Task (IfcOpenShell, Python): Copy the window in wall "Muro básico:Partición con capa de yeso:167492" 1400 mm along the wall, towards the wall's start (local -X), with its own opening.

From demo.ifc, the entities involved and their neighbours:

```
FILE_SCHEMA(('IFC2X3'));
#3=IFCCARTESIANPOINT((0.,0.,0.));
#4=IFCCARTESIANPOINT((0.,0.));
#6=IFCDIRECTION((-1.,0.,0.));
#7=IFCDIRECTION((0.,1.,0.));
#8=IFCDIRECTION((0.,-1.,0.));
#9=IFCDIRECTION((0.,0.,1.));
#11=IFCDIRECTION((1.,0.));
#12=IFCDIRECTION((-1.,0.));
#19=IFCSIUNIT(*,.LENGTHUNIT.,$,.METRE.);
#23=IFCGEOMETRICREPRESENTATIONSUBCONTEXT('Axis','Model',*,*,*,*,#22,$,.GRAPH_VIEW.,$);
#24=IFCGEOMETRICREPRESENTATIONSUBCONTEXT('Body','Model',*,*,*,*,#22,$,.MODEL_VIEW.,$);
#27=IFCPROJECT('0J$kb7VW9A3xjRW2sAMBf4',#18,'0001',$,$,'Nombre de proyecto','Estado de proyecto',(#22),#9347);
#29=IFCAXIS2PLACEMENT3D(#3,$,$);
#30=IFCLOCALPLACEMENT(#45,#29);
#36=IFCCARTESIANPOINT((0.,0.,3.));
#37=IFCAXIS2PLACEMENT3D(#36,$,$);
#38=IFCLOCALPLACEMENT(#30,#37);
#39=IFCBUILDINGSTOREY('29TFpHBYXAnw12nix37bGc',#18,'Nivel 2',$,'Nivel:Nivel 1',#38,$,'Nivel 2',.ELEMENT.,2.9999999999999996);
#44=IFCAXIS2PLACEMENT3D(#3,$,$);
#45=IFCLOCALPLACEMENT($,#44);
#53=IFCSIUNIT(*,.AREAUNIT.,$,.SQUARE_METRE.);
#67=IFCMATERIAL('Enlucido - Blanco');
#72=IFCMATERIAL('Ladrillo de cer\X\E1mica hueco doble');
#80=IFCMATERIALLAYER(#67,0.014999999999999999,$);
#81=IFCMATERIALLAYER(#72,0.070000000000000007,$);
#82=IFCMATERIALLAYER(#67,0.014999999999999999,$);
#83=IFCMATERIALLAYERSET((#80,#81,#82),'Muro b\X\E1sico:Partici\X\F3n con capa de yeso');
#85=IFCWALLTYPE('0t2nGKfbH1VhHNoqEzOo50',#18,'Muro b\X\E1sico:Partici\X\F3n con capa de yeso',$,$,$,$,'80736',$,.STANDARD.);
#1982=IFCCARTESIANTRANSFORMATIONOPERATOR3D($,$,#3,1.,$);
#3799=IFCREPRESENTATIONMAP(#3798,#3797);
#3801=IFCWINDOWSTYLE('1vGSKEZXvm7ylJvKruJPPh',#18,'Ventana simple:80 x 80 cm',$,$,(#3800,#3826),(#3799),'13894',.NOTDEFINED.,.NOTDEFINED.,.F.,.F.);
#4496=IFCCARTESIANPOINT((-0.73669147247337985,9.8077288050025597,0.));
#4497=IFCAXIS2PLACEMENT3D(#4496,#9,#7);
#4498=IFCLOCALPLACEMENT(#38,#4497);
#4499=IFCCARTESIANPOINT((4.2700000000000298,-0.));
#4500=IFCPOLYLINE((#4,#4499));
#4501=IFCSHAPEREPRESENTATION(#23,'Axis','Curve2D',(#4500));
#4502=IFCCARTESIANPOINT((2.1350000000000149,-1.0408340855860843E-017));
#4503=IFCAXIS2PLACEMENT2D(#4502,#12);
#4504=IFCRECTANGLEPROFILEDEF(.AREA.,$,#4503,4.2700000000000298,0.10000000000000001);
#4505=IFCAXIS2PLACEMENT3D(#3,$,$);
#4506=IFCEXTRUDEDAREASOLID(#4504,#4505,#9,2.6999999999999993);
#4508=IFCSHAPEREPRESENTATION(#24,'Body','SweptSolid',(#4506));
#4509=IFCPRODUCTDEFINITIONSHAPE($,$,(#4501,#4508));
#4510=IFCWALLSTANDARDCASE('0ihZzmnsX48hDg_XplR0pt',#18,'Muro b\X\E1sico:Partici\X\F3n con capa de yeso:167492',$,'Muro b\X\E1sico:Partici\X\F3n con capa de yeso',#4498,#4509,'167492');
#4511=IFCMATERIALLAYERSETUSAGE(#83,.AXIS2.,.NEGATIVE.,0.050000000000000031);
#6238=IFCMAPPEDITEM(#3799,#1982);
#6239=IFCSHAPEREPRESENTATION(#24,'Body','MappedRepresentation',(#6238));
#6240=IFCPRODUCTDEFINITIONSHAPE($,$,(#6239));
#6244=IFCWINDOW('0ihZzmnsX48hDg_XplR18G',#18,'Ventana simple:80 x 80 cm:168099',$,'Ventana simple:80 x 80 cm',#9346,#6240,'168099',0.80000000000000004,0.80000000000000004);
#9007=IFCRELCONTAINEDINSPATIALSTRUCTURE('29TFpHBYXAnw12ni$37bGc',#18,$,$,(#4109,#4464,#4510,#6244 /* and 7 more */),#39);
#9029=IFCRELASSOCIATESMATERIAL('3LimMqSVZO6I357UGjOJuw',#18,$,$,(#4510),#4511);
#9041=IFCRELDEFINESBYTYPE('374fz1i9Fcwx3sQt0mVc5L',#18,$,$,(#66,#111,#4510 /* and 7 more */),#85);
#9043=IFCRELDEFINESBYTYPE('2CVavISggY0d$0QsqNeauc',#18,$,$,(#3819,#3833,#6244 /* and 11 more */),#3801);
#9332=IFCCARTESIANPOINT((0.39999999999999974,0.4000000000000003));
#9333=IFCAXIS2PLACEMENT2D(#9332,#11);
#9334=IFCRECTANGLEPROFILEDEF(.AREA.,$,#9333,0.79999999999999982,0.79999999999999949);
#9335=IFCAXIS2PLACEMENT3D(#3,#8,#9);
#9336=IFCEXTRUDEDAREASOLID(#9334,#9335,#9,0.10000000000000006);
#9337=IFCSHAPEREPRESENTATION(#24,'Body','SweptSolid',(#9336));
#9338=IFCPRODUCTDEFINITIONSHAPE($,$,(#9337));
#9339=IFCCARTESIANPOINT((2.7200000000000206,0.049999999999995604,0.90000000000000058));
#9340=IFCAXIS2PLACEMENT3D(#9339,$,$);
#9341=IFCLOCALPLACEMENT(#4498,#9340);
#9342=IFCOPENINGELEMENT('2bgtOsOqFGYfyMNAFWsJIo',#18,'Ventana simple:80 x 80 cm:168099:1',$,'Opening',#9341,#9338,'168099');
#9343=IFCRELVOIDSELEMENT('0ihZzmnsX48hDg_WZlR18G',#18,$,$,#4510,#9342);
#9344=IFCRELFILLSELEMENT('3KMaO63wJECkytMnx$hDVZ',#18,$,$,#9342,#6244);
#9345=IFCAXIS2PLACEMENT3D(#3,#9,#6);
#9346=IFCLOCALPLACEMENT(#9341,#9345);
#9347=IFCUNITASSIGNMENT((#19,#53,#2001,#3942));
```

```python
import ifcopenshell
import ifcopenshell.api.feature
import ifcopenshell.api.geometry
import ifcopenshell.api.root
import ifcopenshell.geom
import ifcopenshell.util.element
import ifcopenshell.util.placement
import ifcopenshell.util.shape
import ifcopenshell.util.unit

model = ifcopenshell.open("demo.ifc")
unit_scale = ifcopenshell.util.unit.calculate_unit_scale(model)
settings = ifcopenshell.geom.settings()


def volume(element):
    """Net volume in cubic metres, openings subtracted."""
    shape = ifcopenshell.geom.create_shape(settings, element)
    return ifcopenshell.util.shape.get_volume(shape.geometry)


def reuse_history(source, copy):
    """copy_class also copies each property set's owner history, people and application; keep the originals."""
    for rel in copy.IsDefinedBy:
        if rel.is_a("IfcRelDefinesByProperties") and (history := rel.RelatingPropertyDefinition.OwnerHistory):
            rel.RelatingPropertyDefinition.OwnerHistory = source.OwnerHistory
            ifcopenshell.util.element.remove_deep2(model, history)


window = model.by_guid("0ihZzmnsX48hDg_XplR18G")
opening = window.FillsVoids[0].RelatingOpeningElement
wall = opening.VoidsElements[0].RelatingBuildingElement
before = volume(wall)
shift = ifcopenshell.util.placement.get_local_placement(wall.ObjectPlacement)[:3, 0] * -1.4 / unit_scale

# copy_class copies the void relationship, type, container and properties, but no geometry.
new_opening = ifcopenshell.api.root.copy_class(model, product=opening)
new_opening.Representation = ifcopenshell.util.element.copy_deep(
    model, opening.Representation, exclude=["IfcGeometricRepresentationContext", "IfcRepresentationMap"]
)
new_opening.Name = "Ventana simple:80 x 80 cm"
new_opening.Tag = None
new_window = ifcopenshell.api.root.copy_class(model, product=window)
new_window.Representation = ifcopenshell.util.element.copy_deep(
    model, window.Representation, exclude=["IfcGeometricRepresentationContext", "IfcRepresentationMap"]
)
new_window.Name = "Ventana simple:80 x 80 cm"
new_window.Tag = None
reuse_history(window, new_window)
fills = ifcopenshell.api.feature.add_filling(model, opening=new_opening, element=new_window)
fills.OwnerHistory = new_window.OwnerHistory  # required in IFC2X3

for old, new in ((opening, new_opening), (window, new_window)):
    matrix = ifcopenshell.util.placement.get_local_placement(old.ObjectPlacement)
    matrix[:3, 3] += shift
    ifcopenshell.api.geometry.edit_object_placement(model, product=new, matrix=matrix, is_si=False)

after = volume(wall)

print(f"wall volume {before:.3f} -> {after:.3f} m3")

model.write("demo_rev.ifc")
```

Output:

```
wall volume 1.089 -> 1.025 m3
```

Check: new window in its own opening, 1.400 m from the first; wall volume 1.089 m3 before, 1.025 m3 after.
